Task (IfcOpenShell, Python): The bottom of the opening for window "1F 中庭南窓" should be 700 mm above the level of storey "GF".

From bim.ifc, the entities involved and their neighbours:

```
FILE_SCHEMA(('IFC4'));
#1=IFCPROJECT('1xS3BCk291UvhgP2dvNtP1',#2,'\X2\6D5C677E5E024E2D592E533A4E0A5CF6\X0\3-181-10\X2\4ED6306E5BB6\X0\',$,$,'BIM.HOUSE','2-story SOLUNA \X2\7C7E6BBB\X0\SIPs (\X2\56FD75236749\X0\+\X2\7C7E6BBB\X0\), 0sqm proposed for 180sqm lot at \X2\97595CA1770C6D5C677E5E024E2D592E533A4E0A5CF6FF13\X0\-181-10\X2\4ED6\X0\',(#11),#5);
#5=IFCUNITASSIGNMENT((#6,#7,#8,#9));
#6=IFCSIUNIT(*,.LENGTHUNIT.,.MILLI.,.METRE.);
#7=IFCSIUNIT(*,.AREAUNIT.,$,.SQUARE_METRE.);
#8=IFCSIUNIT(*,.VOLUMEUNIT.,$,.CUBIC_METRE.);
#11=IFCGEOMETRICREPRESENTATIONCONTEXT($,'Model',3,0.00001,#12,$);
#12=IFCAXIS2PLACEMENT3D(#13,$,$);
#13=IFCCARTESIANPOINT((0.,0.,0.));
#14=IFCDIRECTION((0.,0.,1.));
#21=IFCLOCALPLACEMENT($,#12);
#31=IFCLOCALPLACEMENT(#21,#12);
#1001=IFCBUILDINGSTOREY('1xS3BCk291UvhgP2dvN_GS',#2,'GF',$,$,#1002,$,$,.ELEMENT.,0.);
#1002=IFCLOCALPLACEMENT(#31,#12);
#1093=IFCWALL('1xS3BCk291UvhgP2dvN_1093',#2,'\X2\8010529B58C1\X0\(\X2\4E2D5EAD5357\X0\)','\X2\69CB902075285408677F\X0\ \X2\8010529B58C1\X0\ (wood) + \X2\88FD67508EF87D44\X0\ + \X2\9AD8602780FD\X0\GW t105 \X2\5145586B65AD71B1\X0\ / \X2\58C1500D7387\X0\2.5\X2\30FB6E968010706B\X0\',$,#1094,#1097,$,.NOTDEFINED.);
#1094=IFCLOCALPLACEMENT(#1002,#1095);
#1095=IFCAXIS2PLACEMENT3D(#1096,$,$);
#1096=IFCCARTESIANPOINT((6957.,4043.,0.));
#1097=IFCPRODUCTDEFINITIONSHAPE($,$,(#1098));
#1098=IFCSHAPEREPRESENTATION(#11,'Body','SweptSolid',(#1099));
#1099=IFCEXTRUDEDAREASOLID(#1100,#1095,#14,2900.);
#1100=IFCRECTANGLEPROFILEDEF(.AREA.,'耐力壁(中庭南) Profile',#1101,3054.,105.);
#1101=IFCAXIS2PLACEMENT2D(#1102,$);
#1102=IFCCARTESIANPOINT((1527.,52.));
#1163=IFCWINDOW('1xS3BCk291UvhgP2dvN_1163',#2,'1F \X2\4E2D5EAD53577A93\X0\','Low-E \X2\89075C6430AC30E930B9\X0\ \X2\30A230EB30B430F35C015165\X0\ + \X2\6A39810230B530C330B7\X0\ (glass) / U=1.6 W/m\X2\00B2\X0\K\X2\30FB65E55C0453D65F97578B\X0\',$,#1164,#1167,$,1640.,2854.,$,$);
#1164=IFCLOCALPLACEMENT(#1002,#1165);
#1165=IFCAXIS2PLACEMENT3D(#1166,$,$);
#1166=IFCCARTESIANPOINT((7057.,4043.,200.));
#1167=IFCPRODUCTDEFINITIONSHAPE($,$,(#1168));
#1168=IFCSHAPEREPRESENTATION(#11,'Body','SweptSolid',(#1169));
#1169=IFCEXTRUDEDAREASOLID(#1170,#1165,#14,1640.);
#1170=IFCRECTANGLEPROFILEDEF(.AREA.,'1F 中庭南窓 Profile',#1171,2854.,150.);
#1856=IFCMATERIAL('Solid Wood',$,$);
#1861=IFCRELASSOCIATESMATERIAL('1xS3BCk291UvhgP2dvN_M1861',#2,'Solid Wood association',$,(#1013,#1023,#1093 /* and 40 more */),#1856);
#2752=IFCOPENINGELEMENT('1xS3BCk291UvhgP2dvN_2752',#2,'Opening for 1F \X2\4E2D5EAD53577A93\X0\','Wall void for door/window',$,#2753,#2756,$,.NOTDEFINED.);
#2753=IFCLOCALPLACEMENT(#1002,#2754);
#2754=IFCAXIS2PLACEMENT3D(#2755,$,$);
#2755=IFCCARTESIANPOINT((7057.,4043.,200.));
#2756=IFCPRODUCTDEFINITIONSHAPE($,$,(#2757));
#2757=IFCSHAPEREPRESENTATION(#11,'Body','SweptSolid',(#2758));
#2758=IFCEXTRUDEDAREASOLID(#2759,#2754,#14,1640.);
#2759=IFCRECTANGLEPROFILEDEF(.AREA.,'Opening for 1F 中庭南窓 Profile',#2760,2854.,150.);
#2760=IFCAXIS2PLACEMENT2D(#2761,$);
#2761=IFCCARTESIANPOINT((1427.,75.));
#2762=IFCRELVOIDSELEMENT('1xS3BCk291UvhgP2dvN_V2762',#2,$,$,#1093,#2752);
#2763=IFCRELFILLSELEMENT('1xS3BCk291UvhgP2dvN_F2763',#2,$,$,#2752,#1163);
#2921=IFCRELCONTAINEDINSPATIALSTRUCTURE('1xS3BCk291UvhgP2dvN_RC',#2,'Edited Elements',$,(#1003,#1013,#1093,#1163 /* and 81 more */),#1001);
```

```python
import numpy as np
import ifcopenshell
import ifcopenshell.api.geometry
import ifcopenshell.geom
import ifcopenshell.util.element
import ifcopenshell.util.placement
import ifcopenshell.util.shape
import ifcopenshell.util.unit

model = ifcopenshell.open("bim.ifc")
unit_scale = ifcopenshell.util.unit.calculate_unit_scale(model)

window = model.by_guid("1xS3BCk291UvhgP2dvN_1163")
opening = window.FillsVoids[0].RelatingOpeningElement
storey = ifcopenshell.util.element.get_container(window, ifc_class="IfcBuildingStorey")
level = ifcopenshell.util.placement.get_local_placement(storey.ObjectPlacement)[2, 3]

# The opening's origin need not be at the sill, so measure its lowest point.
shape = ifcopenshell.geom.create_shape(ifcopenshell.geom.settings(), opening)
bottom = ifcopenshell.util.shape.get_shape_bottom_elevation(shape, shape.geometry) / unit_scale
dz = level + 0.7 / unit_scale - bottom

shift = np.array([0.0, 0.0, dz])
# The window is not placed relative to its opening, so move both.
for product in (opening, window):
    matrix = ifcopenshell.util.placement.get_local_placement(product.ObjectPlacement)
    matrix[:3, 3] += shift
    ifcopenshell.api.geometry.edit_object_placement(model, product=product, matrix=matrix, is_si=False)

print(f"moved by {dz * unit_scale:+.3f} m")

model.write("bim_edited.ifc")
```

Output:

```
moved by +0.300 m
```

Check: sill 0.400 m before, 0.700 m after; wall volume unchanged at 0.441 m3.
